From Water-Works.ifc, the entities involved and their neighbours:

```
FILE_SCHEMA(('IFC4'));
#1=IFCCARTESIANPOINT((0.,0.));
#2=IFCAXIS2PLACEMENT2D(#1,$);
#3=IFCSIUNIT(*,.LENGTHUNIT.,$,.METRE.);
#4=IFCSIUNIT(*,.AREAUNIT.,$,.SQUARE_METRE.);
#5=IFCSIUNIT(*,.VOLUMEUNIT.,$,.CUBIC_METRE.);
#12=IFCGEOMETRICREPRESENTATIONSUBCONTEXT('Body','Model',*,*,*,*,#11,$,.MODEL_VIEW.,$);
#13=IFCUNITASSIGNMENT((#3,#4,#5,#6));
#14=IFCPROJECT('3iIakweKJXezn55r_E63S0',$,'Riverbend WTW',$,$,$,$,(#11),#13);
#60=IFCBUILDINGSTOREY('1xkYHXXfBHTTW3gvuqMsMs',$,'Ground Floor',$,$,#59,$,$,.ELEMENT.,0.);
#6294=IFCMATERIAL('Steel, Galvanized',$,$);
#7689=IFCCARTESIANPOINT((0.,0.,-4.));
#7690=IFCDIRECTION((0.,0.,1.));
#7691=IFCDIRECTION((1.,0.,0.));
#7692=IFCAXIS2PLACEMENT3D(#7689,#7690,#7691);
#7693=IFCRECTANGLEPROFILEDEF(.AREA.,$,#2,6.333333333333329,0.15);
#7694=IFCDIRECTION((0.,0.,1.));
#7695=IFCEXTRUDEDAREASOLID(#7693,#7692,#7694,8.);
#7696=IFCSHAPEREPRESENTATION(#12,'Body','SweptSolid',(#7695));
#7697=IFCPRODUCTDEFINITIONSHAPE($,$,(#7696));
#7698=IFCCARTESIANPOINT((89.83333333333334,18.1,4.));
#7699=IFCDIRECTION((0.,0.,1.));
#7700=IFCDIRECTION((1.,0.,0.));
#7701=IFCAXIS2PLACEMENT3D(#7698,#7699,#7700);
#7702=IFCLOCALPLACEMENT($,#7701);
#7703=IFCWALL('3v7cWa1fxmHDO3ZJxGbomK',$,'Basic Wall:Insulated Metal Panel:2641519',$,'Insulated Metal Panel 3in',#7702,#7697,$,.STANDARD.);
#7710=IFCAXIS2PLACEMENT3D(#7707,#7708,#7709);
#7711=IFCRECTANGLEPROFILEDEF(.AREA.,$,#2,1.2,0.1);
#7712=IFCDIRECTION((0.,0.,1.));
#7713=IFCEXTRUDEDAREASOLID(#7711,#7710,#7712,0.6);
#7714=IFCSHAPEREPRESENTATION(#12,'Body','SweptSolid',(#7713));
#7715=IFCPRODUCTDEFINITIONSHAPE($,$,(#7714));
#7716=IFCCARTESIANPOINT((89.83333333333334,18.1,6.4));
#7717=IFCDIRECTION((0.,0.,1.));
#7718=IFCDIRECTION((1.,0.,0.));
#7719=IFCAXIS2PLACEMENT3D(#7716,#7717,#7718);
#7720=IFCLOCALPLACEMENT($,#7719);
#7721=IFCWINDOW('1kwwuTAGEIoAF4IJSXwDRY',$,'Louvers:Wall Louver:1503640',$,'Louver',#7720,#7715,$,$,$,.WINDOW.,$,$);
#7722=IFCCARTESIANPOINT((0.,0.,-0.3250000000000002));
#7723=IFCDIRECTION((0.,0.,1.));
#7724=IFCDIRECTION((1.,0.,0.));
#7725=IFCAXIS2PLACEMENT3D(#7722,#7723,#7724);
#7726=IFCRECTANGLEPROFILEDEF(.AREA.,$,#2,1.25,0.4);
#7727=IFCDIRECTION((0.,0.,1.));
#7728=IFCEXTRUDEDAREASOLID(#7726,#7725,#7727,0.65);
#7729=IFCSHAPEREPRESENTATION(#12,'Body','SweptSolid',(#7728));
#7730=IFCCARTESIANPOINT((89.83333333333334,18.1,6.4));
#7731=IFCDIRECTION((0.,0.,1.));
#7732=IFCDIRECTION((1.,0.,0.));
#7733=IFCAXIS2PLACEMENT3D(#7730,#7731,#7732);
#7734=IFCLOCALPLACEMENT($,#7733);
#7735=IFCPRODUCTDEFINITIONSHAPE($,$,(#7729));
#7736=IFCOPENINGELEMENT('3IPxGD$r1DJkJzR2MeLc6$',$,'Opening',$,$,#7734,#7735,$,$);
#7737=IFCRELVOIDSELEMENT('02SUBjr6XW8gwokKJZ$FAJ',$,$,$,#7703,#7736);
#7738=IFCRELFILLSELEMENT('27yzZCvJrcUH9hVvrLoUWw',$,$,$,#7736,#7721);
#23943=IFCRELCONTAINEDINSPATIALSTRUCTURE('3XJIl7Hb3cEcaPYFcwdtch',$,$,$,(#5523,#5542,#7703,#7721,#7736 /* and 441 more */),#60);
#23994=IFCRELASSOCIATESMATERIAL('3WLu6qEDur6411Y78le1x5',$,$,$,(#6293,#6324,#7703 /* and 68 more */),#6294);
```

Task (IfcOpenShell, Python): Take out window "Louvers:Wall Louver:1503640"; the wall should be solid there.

```python
import ifcopenshell
import ifcopenshell.api.feature
import ifcopenshell.api.root
import ifcopenshell.geom
import ifcopenshell.util.shape

model = ifcopenshell.open("Water-Works.ifc")
settings = ifcopenshell.geom.settings()


def volume(element):
    """Net volume in cubic metres, openings subtracted."""
    shape = ifcopenshell.geom.create_shape(settings, element)
    return ifcopenshell.util.shape.get_volume(shape.geometry)


window = model.by_guid("1kwwuTAGEIoAF4IJSXwDRY")
opening = window.FillsVoids[0].RelatingOpeningElement
wall = opening.VoidsElements[0].RelatingBuildingElement
before = volume(wall)

ifcopenshell.api.root.remove_product(model, product=window)
ifcopenshell.api.feature.remove_feature(model, feature=opening)

after = volume(wall)

print(f"wall volume {before:.3f} -> {after:.3f} m3")

model.write("Water-Works_updated.ifc")
```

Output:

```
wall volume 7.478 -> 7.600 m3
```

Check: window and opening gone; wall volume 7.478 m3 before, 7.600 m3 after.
